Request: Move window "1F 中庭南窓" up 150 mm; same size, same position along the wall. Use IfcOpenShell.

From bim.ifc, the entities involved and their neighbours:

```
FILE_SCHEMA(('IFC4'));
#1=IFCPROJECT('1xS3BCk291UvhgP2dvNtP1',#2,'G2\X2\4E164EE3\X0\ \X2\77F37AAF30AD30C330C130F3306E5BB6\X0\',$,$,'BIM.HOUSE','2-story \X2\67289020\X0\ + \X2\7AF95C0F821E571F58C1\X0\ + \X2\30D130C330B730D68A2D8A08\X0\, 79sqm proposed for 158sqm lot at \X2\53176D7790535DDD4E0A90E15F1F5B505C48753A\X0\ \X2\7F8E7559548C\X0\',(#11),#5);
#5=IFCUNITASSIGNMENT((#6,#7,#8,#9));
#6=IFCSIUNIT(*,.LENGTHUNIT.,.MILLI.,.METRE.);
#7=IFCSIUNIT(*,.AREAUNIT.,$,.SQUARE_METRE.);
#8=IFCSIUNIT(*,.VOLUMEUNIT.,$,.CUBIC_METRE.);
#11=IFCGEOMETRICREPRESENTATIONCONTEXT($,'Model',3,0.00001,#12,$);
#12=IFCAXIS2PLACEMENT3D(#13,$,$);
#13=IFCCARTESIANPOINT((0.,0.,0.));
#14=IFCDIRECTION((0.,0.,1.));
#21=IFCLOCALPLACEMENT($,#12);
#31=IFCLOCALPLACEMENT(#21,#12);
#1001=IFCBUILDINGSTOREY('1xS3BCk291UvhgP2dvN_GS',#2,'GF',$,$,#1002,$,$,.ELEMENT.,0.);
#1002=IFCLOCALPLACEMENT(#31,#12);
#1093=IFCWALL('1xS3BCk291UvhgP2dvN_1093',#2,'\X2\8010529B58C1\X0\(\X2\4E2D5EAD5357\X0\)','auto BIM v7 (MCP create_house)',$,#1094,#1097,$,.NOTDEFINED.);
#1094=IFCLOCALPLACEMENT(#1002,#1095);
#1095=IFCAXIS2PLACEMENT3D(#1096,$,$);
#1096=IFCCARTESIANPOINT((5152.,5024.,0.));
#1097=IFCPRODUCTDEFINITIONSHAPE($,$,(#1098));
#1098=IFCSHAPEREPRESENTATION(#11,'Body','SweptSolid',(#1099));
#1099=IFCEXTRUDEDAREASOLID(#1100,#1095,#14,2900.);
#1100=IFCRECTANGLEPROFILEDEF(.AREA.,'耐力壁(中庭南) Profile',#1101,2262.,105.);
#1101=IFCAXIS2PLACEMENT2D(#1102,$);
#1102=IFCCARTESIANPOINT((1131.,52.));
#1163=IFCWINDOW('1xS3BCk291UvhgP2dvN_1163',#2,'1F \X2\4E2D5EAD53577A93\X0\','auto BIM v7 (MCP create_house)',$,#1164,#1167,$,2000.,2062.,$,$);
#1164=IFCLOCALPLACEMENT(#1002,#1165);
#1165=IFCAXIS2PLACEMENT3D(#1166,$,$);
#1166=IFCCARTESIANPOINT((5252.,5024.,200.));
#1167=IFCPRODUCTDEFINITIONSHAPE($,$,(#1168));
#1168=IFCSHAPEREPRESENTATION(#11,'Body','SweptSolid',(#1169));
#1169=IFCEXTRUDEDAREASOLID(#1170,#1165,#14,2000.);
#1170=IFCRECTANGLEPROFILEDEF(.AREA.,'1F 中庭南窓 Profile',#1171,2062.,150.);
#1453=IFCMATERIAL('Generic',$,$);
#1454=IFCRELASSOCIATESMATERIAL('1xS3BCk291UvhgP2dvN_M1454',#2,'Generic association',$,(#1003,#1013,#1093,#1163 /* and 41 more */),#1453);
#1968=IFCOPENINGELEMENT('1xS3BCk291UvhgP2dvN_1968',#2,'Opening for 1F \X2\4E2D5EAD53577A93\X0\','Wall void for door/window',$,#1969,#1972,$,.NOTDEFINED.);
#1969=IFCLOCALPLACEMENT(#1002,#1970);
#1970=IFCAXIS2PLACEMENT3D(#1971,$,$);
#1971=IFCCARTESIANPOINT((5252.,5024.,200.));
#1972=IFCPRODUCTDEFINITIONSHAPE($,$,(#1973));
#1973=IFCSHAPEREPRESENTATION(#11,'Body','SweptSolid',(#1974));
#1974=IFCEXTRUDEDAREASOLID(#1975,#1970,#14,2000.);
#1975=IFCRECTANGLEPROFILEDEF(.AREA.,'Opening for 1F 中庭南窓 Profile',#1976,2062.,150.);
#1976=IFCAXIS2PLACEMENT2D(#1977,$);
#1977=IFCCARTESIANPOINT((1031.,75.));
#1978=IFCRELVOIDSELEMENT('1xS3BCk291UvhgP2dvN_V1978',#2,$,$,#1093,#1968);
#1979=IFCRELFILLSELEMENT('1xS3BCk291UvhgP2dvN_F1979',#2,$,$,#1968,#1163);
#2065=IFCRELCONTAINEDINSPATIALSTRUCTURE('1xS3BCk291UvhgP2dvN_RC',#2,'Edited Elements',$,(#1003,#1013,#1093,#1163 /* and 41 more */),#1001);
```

```python
import numpy as np
import ifcopenshell
import ifcopenshell.api.geometry
import ifcopenshell.util.placement
import ifcopenshell.util.unit

model = ifcopenshell.open("bim.ifc")
unit_scale = ifcopenshell.util.unit.calculate_unit_scale(model)

window = model.by_id(1163)
opening = window.FillsVoids[0].RelatingOpeningElement
dz = 150.0

shift = np.array([0.0, 0.0, dz])
# The window is not placed relative to its opening, so move both.
for product in (opening, window):
    matrix = ifcopenshell.util.placement.get_local_placement(product.ObjectPlacement)
    matrix[:3, 3] += shift
    ifcopenshell.api.geometry.edit_object_placement(model, product=product, matrix=matrix, is_si=False)

print(f"moved by {dz * unit_scale:+.3f} m")

model.write("bim_v2.ifc")
```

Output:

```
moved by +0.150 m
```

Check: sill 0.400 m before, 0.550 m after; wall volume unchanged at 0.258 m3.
